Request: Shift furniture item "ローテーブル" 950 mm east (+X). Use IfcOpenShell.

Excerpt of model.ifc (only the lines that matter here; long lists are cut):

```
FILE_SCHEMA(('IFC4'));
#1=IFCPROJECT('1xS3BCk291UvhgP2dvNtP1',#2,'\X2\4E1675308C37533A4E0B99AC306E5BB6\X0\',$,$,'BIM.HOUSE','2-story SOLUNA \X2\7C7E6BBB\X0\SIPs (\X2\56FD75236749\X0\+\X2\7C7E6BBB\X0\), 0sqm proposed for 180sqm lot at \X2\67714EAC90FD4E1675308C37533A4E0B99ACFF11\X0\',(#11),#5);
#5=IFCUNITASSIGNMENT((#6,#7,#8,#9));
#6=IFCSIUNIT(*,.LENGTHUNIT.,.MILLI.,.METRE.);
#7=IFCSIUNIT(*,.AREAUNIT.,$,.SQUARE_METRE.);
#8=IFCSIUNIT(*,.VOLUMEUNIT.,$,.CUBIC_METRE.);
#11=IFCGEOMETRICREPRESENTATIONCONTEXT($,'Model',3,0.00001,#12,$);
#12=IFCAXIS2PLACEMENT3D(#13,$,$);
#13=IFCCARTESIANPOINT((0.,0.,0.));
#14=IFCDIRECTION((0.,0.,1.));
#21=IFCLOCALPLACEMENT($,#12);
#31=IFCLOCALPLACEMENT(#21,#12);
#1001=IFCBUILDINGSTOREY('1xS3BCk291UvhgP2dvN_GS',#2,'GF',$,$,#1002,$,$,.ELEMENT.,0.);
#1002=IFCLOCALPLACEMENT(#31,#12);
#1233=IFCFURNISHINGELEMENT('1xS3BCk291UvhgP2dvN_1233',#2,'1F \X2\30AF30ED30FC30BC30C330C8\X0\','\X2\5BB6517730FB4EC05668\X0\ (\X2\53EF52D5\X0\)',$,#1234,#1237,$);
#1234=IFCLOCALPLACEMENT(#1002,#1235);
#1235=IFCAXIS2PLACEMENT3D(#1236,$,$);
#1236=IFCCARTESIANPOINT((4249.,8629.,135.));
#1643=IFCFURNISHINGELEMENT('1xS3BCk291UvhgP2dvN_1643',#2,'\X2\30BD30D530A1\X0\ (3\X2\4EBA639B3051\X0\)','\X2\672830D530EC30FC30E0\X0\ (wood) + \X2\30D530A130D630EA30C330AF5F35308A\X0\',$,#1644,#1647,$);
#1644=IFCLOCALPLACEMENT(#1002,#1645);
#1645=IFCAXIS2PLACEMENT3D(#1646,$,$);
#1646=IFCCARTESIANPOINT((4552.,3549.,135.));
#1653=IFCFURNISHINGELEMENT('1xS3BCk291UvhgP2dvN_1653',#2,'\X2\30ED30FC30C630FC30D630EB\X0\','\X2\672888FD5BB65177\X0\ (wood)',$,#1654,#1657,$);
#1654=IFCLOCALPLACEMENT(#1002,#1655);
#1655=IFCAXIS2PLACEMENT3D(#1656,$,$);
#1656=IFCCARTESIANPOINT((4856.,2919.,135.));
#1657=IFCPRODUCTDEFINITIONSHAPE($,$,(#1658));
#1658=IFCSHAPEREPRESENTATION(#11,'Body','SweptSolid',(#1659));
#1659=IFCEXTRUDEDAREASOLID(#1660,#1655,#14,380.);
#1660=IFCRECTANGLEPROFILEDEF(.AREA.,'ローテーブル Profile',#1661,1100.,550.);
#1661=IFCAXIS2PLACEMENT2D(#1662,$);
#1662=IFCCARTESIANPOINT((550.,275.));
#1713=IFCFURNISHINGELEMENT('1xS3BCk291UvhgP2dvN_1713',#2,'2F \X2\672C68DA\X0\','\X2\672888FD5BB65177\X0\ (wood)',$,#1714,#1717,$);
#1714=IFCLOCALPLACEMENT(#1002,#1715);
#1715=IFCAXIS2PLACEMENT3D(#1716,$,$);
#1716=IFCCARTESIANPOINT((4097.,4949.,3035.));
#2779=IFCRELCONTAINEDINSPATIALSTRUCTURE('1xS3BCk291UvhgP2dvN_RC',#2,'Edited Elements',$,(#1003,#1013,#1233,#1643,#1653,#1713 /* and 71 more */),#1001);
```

```python
import ifcopenshell
import ifcopenshell.api.geometry
import ifcopenshell.util.placement
import ifcopenshell.util.unit

model = ifcopenshell.open("model.ifc")
unit_scale = ifcopenshell.util.unit.calculate_unit_scale(model)

item = model.by_guid("1xS3BCk291UvhgP2dvN_1653")
matrix = ifcopenshell.util.placement.get_local_placement(item.ObjectPlacement)
matrix[0, 3] += 0.95 / unit_scale
ifcopenshell.api.geometry.edit_object_placement(model, product=item, matrix=matrix, is_si=False)

print(ifcopenshell.util.placement.get_local_placement(item.ObjectPlacement).round(3) + 0.0)

model.write("model_edited.ifc")
```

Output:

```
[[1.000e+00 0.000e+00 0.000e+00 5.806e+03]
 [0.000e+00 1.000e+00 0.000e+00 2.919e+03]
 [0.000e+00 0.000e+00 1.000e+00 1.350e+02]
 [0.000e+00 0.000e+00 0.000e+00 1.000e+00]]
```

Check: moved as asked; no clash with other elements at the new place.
